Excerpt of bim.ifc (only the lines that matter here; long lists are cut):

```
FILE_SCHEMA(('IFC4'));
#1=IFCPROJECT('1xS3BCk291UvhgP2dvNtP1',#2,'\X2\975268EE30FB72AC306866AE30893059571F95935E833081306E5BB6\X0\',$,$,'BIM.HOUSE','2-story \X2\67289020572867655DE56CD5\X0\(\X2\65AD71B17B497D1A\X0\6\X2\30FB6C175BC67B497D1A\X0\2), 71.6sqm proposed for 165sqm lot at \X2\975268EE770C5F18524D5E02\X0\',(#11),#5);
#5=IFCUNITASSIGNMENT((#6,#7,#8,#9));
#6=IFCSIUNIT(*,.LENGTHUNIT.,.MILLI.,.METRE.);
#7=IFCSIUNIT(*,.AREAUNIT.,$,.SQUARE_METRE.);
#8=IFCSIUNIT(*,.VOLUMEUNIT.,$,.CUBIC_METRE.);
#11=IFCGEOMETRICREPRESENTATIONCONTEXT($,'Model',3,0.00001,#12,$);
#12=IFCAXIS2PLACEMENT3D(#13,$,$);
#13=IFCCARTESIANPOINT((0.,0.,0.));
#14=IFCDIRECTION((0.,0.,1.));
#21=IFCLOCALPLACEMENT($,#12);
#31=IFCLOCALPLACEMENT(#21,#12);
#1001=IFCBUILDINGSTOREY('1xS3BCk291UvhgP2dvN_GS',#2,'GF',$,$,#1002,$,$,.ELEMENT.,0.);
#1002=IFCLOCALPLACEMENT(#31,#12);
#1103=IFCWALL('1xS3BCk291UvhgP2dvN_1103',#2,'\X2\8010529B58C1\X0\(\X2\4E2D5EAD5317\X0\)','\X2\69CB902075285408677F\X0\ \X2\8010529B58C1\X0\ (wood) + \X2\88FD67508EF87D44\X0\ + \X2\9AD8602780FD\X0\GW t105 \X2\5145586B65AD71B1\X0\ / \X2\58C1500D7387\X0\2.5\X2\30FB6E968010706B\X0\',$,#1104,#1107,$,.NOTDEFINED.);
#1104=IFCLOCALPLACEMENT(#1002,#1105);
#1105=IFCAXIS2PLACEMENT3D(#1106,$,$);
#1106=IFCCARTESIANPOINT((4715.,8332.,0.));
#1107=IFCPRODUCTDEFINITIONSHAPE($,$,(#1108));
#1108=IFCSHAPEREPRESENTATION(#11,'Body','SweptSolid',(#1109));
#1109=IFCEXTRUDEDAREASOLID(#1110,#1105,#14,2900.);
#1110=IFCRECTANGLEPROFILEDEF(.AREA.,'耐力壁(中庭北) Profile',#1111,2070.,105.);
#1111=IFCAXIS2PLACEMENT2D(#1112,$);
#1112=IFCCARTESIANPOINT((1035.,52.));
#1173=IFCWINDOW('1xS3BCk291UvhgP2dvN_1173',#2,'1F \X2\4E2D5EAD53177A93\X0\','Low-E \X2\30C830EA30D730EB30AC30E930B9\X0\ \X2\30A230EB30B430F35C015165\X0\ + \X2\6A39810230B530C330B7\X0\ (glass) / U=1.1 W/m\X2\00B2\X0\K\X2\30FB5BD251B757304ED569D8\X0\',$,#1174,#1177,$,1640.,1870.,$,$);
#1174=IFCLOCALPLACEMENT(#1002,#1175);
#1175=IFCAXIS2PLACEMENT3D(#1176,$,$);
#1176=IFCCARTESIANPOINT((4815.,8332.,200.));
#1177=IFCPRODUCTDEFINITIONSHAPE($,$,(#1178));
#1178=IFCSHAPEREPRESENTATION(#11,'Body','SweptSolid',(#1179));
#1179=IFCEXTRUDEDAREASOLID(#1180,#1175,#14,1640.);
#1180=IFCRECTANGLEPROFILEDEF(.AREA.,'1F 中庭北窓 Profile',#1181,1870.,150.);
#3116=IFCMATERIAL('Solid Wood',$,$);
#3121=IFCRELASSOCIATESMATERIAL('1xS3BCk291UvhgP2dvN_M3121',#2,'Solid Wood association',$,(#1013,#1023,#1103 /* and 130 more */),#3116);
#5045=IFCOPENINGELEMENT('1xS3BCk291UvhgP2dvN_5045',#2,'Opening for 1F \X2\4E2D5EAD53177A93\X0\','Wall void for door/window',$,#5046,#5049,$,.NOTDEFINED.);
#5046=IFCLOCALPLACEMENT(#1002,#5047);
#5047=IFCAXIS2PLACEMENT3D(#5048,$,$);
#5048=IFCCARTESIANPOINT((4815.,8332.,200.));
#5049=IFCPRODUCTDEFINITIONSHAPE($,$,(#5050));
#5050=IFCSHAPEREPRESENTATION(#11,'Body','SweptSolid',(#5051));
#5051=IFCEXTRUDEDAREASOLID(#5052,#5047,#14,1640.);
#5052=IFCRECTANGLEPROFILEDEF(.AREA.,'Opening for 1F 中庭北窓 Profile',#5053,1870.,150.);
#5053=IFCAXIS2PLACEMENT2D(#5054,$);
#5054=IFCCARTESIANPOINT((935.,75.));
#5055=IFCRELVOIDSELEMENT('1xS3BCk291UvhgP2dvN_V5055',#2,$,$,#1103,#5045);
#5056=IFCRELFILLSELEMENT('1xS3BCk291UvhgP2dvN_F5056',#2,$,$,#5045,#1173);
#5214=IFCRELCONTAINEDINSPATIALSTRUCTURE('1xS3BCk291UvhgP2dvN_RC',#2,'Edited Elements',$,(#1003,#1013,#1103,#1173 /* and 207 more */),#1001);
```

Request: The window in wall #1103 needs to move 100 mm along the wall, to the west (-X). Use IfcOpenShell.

```python
import ifcopenshell
import ifcopenshell.api.geometry
import ifcopenshell.util.placement
import ifcopenshell.util.unit

model = ifcopenshell.open("bim.ifc")
unit_scale = ifcopenshell.util.unit.calculate_unit_scale(model)

window = model.by_guid("1xS3BCk291UvhgP2dvN_1173")
opening = window.FillsVoids[0].RelatingOpeningElement
wall = opening.VoidsElements[0].RelatingBuildingElement

wall_matrix = ifcopenshell.util.placement.get_local_placement(wall.ObjectPlacement)
shift = wall_matrix[:3, 0] * -0.1 / unit_scale
before = ifcopenshell.util.placement.get_local_placement(window.ObjectPlacement)[:3, 3].copy()

# The window is not placed relative to its opening, so move both.
for product in (opening, window):
    matrix = ifcopenshell.util.placement.get_local_placement(product.ObjectPlacement)
    matrix[:3, 3] += shift
    ifcopenshell.api.geometry.edit_object_placement(model, product=product, matrix=matrix, is_si=False)

after = ifcopenshell.util.placement.get_local_placement(window.ObjectPlacement)[:3, 3]
print("window moved by", (after - before).round(3) + 0.0)

model.write("bim_edited.ifc")
```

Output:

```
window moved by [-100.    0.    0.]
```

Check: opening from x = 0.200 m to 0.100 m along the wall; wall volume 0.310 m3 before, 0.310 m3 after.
